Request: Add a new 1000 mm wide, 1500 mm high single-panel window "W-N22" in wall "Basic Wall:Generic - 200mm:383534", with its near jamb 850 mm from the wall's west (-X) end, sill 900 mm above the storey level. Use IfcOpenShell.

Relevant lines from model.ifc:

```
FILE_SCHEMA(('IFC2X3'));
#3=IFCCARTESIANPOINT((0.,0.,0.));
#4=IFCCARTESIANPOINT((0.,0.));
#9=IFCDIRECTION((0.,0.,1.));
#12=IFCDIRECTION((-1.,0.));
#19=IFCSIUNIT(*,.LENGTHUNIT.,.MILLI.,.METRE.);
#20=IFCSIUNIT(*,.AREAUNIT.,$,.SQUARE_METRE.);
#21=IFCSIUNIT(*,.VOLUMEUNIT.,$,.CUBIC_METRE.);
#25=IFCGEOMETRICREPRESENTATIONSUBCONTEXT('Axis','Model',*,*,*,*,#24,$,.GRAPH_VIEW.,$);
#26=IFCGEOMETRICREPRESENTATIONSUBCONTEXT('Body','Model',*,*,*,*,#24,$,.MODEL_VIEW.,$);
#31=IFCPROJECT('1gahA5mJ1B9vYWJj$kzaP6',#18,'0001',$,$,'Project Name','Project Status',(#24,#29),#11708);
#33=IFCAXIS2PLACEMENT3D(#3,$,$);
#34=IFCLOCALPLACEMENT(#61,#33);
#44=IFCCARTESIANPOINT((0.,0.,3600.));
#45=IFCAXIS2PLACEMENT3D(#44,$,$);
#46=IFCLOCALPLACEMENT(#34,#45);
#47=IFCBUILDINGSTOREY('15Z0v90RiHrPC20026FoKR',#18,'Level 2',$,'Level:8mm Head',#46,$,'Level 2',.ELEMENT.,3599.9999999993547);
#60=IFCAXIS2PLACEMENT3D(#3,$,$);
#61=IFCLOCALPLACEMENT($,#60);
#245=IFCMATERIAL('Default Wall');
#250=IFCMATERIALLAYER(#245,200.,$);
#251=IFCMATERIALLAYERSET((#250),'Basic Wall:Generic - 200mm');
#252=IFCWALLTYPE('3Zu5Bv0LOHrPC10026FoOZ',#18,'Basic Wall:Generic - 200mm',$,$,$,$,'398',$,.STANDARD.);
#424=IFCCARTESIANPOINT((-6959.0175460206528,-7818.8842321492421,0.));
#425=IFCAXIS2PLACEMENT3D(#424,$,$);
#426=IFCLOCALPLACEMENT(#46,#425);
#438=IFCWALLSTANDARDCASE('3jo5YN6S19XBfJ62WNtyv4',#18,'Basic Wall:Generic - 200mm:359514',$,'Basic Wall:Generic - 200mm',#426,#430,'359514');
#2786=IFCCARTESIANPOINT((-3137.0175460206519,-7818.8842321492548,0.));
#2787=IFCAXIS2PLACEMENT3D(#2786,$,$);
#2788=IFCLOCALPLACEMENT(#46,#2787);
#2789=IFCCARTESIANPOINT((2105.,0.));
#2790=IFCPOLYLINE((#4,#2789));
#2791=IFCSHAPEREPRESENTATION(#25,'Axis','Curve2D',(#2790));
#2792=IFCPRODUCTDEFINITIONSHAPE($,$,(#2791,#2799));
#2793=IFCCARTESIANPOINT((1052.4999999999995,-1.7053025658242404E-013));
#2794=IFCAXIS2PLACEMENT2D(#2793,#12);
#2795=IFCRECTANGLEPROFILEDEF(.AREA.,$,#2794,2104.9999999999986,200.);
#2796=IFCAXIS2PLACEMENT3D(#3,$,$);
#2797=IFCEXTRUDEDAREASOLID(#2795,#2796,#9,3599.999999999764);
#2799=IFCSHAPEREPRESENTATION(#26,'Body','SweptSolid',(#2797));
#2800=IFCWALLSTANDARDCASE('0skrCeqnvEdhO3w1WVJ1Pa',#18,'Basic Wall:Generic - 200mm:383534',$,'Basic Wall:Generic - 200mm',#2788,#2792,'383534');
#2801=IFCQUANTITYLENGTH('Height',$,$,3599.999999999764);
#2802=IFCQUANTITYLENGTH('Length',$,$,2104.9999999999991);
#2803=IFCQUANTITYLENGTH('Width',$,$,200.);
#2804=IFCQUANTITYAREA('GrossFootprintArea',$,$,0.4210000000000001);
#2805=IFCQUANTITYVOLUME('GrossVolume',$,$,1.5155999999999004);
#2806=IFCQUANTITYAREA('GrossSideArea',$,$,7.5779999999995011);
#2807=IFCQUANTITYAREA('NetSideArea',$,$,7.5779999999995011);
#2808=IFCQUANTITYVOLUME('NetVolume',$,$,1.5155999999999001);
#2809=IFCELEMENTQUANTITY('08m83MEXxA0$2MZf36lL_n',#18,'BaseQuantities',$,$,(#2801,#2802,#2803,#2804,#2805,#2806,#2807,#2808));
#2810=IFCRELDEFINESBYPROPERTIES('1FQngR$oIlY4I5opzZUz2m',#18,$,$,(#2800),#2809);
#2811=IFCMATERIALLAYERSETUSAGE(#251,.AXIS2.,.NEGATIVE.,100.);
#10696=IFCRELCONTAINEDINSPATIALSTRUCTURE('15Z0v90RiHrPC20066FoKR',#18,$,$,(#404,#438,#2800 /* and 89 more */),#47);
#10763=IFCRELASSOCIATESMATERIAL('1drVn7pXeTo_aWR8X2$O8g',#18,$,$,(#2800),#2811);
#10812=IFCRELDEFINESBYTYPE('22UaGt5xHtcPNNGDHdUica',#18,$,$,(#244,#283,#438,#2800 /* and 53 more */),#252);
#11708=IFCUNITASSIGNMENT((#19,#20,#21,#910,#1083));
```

```python
import numpy as np
import ifcopenshell
import ifcopenshell.api.feature
import ifcopenshell.api.geometry
import ifcopenshell.api.pset
import ifcopenshell.api.root
import ifcopenshell.api.spatial
import ifcopenshell.api.type
import ifcopenshell.geom
import ifcopenshell.util.element
import ifcopenshell.util.placement
import ifcopenshell.util.representation
import ifcopenshell.util.shape
import ifcopenshell.util.unit

model = ifcopenshell.open("model.ifc")
unit_scale = ifcopenshell.util.unit.calculate_unit_scale(model)
area_scale = ifcopenshell.util.unit.calculate_unit_scale(model, "AREAUNIT")
volume_scale = ifcopenshell.util.unit.calculate_unit_scale(model, "VOLUMEUNIT")
settings = ifcopenshell.geom.settings()


def volume(element):
    """Net volume in cubic metres, openings subtracted."""
    shape = ifcopenshell.geom.create_shape(settings, element)
    return ifcopenshell.util.shape.get_volume(shape.geometry)


wall = model.by_guid("0skrCeqnvEdhO3w1WVJ1Pa")
storey = ifcopenshell.util.element.get_container(wall, ifc_class="IfcBuildingStorey")
context = ifcopenshell.util.representation.get_context(model, "Model", "Body", "MODEL_VIEW")
before = volume(wall)

width, height, from_end, sill = 1, 1.5, 0.85, 0.9  # metres

# The wall runs along its own X axis, and the end named is its -X end.
wall_shape = ifcopenshell.geom.create_shape(settings, wall)
x, y, z = ifcopenshell.util.shape.get_vertices(wall_shape.geometry).T
start = x.min() + from_end
face, thickness = float(y.min()), float(y.max() - y.min())
wall_matrix = ifcopenshell.util.placement.get_local_placement(wall.ObjectPlacement)
level = ifcopenshell.util.placement.get_local_placement(storey.ObjectPlacement)[2, 3]


def in_wall(x, y):
    """Placement at x, y metres in the wall's axes, at sill height."""
    matrix = wall_matrix.copy()
    matrix[:, 3] = wall_matrix @ np.array([x / unit_scale, y / unit_scale, 0.0, 1.0])
    matrix[2, 3] = level + sill / unit_scale
    return matrix


# Opening: a box that overshoots both wall faces by 50 mm.
opening = ifcopenshell.api.root.create_entity(model, ifc_class="IfcOpeningElement")
box = ifcopenshell.api.geometry.add_wall_representation(
    model, context=context, length=width, height=height, thickness=thickness + 0.1
)
ifcopenshell.api.geometry.assign_representation(model, product=opening, representation=box)
ifcopenshell.api.geometry.edit_object_placement(model, product=opening, matrix=in_wall(start, face - 0.05), is_si=False)
ifcopenshell.api.feature.add_feature(model, feature=opening, element=wall)

window = ifcopenshell.api.root.create_entity(model, ifc_class="IfcWindow", name="W-N22")
window.OverallWidth, window.OverallHeight = width / unit_scale, height / unit_scale
body = ifcopenshell.api.geometry.add_window_representation(
    model,
    context=context,
    overall_width=window.OverallWidth,
    overall_height=window.OverallHeight,
    partition_type="SINGLE_PANEL",
)
ifcopenshell.api.geometry.assign_representation(model, product=window, representation=body)
ifcopenshell.api.spatial.assign_container(model, products=[window], relating_structure=storey)
fills = ifcopenshell.api.feature.add_filling(model, opening=opening, element=window)
fills.OwnerHistory = window.OwnerHistory  # required in IFC2X3

# IFC2X3 keeps the operation on the window style.
style = ifcopenshell.api.root.create_entity(model, ifc_class="IfcWindowStyle", name="W-N22")
style.OperationType, style.ConstructionType = "SINGLE_PANEL", "NOTDEFINED"
style.ParameterTakesPrecedence = style.Sizeable = False
ifcopenshell.api.type.assign_type(model, related_objects=[window], relating_type=style)

# Centre the window in the wall's thickness.
ifcopenshell.api.geometry.edit_object_placement(model, product=window, matrix=in_wall(start, face), is_si=False)
window_shape = ifcopenshell.geom.create_shape(settings, window)
depth = ifcopenshell.util.shape.get_vertices(window_shape.geometry)[:, 1]
offset = face + thickness / 2 - (depth.min() + depth.max()) / 2
ifcopenshell.api.geometry.edit_object_placement(model, product=window, matrix=in_wall(start, offset), is_si=False)

after = volume(wall)

# Update the wall's stored quantities.
qto = model.by_id(ifcopenshell.util.element.get_pset(wall, "BaseQuantities", should_inherit=False)["id"])
ifcopenshell.api.pset.edit_qto(model, qto=qto, properties={
    "NetSideArea": after / thickness / area_scale,
    "NetVolume": after / volume_scale,
})

print(f"wall volume {before:.3f} -> {after:.3f} m3")

model.write("model_updated.ifc")
```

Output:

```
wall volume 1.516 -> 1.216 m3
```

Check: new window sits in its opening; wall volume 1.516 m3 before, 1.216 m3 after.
